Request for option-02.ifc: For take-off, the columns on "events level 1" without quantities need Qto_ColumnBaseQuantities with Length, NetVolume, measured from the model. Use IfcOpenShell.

First a look at what the model holds.

```python
import ifcopenshell
import ifcopenshell.util.element
import ifcopenshell.util.unit

model = ifcopenshell.open("option-02.ifc")
print(model.schema)
for unit_type in ("LENGTHUNIT", "AREAUNIT", "VOLUMEUNIT"):
    print(unit_type, ifcopenshell.util.unit.calculate_unit_scale(model, unit_type))
storey = next(s for s in model.by_type("IfcBuildingStorey") if s.Name == "events level 1")
columns = [e for e in ifcopenshell.util.element.get_decomposition(storey) if e.is_a("IfcColumn")]
for e in sorted(columns, key=lambda e: e.id()):
    print(e.id(), e.is_a(), e.Name, list(ifcopenshell.util.element.get_psets(e, qtos_only=True)), sep=" | ")
```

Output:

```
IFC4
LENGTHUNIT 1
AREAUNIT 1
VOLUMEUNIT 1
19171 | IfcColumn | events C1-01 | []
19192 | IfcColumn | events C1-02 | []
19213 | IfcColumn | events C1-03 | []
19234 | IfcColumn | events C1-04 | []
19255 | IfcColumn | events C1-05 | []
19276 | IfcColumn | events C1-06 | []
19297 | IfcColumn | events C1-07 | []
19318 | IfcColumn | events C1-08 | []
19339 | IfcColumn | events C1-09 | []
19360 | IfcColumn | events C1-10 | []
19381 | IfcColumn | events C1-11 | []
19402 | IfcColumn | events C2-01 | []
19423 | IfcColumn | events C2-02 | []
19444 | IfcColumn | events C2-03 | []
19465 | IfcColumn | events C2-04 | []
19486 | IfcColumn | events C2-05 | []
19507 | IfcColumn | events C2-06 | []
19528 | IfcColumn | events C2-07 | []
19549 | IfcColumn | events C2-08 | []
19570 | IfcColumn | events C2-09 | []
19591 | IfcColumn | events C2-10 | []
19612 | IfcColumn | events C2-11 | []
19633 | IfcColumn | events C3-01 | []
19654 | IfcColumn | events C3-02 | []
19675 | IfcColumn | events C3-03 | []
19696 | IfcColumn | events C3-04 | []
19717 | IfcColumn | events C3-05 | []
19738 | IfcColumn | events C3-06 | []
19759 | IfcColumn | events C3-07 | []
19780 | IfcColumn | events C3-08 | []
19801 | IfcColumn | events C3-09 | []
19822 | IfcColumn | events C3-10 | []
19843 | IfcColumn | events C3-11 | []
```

```python
import ifcopenshell
import ifcopenshell.api.pset
import ifcopenshell.geom
import ifcopenshell.util.element
import ifcopenshell.util.shape
import ifcopenshell.util.unit

model = ifcopenshell.open("option-02.ifc")
unit_scale = ifcopenshell.util.unit.calculate_unit_scale(model)
volume_scale = ifcopenshell.util.unit.calculate_unit_scale(model, "VOLUMEUNIT")
settings = ifcopenshell.geom.settings()

storey = next(s for s in model.by_type("IfcBuildingStorey") if s.Name == "events level 1")
columns = [e for e in ifcopenshell.util.element.get_decomposition(storey) if e.is_a("IfcColumn")]

for e in sorted(columns, key=lambda e: e.id()):
    if ifcopenshell.util.element.get_psets(e, qtos_only=True, should_inherit=False):
        continue
    # Geometry comes back in metres, in the element's own axes.
    shape = ifcopenshell.geom.create_shape(settings, e)
    values = {
        "Length": ifcopenshell.util.shape.get_z(shape.geometry) / unit_scale,
        "NetVolume": ifcopenshell.util.shape.get_volume(shape.geometry) / volume_scale,
    }
    qto = ifcopenshell.api.pset.add_qto(model, product=e, name="Qto_ColumnBaseQuantities")
    ifcopenshell.api.pset.edit_qto(model, qto=qto, properties=values)
    print(e.id(), {k: round(v, 3) for k, v in values.items()})

model.write("option-02_updated.ifc")
```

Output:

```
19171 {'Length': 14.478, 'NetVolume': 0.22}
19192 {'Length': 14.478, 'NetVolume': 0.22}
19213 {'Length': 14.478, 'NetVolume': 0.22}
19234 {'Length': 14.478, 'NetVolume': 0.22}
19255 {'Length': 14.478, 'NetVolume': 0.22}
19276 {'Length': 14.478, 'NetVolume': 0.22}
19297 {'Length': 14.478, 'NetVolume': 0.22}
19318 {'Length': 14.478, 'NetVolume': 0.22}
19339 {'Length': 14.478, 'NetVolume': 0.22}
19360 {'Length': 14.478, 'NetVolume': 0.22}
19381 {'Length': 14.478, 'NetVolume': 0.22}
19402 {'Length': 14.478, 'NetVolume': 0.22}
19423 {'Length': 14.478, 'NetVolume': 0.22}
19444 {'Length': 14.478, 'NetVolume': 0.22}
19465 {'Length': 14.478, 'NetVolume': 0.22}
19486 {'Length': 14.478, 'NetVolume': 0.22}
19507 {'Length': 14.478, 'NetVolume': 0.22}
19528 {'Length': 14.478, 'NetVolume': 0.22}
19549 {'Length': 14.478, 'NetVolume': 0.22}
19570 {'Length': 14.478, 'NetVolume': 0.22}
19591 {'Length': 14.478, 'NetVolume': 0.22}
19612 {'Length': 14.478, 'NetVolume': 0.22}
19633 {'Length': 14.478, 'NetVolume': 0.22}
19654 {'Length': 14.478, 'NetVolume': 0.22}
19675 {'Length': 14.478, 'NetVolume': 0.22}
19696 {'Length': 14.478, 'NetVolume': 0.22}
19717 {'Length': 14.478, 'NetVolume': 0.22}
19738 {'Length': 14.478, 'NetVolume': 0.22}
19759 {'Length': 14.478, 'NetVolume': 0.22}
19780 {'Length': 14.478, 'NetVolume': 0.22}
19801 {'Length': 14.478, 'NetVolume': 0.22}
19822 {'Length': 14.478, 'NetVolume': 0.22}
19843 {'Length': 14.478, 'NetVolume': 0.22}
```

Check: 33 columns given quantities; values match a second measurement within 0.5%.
